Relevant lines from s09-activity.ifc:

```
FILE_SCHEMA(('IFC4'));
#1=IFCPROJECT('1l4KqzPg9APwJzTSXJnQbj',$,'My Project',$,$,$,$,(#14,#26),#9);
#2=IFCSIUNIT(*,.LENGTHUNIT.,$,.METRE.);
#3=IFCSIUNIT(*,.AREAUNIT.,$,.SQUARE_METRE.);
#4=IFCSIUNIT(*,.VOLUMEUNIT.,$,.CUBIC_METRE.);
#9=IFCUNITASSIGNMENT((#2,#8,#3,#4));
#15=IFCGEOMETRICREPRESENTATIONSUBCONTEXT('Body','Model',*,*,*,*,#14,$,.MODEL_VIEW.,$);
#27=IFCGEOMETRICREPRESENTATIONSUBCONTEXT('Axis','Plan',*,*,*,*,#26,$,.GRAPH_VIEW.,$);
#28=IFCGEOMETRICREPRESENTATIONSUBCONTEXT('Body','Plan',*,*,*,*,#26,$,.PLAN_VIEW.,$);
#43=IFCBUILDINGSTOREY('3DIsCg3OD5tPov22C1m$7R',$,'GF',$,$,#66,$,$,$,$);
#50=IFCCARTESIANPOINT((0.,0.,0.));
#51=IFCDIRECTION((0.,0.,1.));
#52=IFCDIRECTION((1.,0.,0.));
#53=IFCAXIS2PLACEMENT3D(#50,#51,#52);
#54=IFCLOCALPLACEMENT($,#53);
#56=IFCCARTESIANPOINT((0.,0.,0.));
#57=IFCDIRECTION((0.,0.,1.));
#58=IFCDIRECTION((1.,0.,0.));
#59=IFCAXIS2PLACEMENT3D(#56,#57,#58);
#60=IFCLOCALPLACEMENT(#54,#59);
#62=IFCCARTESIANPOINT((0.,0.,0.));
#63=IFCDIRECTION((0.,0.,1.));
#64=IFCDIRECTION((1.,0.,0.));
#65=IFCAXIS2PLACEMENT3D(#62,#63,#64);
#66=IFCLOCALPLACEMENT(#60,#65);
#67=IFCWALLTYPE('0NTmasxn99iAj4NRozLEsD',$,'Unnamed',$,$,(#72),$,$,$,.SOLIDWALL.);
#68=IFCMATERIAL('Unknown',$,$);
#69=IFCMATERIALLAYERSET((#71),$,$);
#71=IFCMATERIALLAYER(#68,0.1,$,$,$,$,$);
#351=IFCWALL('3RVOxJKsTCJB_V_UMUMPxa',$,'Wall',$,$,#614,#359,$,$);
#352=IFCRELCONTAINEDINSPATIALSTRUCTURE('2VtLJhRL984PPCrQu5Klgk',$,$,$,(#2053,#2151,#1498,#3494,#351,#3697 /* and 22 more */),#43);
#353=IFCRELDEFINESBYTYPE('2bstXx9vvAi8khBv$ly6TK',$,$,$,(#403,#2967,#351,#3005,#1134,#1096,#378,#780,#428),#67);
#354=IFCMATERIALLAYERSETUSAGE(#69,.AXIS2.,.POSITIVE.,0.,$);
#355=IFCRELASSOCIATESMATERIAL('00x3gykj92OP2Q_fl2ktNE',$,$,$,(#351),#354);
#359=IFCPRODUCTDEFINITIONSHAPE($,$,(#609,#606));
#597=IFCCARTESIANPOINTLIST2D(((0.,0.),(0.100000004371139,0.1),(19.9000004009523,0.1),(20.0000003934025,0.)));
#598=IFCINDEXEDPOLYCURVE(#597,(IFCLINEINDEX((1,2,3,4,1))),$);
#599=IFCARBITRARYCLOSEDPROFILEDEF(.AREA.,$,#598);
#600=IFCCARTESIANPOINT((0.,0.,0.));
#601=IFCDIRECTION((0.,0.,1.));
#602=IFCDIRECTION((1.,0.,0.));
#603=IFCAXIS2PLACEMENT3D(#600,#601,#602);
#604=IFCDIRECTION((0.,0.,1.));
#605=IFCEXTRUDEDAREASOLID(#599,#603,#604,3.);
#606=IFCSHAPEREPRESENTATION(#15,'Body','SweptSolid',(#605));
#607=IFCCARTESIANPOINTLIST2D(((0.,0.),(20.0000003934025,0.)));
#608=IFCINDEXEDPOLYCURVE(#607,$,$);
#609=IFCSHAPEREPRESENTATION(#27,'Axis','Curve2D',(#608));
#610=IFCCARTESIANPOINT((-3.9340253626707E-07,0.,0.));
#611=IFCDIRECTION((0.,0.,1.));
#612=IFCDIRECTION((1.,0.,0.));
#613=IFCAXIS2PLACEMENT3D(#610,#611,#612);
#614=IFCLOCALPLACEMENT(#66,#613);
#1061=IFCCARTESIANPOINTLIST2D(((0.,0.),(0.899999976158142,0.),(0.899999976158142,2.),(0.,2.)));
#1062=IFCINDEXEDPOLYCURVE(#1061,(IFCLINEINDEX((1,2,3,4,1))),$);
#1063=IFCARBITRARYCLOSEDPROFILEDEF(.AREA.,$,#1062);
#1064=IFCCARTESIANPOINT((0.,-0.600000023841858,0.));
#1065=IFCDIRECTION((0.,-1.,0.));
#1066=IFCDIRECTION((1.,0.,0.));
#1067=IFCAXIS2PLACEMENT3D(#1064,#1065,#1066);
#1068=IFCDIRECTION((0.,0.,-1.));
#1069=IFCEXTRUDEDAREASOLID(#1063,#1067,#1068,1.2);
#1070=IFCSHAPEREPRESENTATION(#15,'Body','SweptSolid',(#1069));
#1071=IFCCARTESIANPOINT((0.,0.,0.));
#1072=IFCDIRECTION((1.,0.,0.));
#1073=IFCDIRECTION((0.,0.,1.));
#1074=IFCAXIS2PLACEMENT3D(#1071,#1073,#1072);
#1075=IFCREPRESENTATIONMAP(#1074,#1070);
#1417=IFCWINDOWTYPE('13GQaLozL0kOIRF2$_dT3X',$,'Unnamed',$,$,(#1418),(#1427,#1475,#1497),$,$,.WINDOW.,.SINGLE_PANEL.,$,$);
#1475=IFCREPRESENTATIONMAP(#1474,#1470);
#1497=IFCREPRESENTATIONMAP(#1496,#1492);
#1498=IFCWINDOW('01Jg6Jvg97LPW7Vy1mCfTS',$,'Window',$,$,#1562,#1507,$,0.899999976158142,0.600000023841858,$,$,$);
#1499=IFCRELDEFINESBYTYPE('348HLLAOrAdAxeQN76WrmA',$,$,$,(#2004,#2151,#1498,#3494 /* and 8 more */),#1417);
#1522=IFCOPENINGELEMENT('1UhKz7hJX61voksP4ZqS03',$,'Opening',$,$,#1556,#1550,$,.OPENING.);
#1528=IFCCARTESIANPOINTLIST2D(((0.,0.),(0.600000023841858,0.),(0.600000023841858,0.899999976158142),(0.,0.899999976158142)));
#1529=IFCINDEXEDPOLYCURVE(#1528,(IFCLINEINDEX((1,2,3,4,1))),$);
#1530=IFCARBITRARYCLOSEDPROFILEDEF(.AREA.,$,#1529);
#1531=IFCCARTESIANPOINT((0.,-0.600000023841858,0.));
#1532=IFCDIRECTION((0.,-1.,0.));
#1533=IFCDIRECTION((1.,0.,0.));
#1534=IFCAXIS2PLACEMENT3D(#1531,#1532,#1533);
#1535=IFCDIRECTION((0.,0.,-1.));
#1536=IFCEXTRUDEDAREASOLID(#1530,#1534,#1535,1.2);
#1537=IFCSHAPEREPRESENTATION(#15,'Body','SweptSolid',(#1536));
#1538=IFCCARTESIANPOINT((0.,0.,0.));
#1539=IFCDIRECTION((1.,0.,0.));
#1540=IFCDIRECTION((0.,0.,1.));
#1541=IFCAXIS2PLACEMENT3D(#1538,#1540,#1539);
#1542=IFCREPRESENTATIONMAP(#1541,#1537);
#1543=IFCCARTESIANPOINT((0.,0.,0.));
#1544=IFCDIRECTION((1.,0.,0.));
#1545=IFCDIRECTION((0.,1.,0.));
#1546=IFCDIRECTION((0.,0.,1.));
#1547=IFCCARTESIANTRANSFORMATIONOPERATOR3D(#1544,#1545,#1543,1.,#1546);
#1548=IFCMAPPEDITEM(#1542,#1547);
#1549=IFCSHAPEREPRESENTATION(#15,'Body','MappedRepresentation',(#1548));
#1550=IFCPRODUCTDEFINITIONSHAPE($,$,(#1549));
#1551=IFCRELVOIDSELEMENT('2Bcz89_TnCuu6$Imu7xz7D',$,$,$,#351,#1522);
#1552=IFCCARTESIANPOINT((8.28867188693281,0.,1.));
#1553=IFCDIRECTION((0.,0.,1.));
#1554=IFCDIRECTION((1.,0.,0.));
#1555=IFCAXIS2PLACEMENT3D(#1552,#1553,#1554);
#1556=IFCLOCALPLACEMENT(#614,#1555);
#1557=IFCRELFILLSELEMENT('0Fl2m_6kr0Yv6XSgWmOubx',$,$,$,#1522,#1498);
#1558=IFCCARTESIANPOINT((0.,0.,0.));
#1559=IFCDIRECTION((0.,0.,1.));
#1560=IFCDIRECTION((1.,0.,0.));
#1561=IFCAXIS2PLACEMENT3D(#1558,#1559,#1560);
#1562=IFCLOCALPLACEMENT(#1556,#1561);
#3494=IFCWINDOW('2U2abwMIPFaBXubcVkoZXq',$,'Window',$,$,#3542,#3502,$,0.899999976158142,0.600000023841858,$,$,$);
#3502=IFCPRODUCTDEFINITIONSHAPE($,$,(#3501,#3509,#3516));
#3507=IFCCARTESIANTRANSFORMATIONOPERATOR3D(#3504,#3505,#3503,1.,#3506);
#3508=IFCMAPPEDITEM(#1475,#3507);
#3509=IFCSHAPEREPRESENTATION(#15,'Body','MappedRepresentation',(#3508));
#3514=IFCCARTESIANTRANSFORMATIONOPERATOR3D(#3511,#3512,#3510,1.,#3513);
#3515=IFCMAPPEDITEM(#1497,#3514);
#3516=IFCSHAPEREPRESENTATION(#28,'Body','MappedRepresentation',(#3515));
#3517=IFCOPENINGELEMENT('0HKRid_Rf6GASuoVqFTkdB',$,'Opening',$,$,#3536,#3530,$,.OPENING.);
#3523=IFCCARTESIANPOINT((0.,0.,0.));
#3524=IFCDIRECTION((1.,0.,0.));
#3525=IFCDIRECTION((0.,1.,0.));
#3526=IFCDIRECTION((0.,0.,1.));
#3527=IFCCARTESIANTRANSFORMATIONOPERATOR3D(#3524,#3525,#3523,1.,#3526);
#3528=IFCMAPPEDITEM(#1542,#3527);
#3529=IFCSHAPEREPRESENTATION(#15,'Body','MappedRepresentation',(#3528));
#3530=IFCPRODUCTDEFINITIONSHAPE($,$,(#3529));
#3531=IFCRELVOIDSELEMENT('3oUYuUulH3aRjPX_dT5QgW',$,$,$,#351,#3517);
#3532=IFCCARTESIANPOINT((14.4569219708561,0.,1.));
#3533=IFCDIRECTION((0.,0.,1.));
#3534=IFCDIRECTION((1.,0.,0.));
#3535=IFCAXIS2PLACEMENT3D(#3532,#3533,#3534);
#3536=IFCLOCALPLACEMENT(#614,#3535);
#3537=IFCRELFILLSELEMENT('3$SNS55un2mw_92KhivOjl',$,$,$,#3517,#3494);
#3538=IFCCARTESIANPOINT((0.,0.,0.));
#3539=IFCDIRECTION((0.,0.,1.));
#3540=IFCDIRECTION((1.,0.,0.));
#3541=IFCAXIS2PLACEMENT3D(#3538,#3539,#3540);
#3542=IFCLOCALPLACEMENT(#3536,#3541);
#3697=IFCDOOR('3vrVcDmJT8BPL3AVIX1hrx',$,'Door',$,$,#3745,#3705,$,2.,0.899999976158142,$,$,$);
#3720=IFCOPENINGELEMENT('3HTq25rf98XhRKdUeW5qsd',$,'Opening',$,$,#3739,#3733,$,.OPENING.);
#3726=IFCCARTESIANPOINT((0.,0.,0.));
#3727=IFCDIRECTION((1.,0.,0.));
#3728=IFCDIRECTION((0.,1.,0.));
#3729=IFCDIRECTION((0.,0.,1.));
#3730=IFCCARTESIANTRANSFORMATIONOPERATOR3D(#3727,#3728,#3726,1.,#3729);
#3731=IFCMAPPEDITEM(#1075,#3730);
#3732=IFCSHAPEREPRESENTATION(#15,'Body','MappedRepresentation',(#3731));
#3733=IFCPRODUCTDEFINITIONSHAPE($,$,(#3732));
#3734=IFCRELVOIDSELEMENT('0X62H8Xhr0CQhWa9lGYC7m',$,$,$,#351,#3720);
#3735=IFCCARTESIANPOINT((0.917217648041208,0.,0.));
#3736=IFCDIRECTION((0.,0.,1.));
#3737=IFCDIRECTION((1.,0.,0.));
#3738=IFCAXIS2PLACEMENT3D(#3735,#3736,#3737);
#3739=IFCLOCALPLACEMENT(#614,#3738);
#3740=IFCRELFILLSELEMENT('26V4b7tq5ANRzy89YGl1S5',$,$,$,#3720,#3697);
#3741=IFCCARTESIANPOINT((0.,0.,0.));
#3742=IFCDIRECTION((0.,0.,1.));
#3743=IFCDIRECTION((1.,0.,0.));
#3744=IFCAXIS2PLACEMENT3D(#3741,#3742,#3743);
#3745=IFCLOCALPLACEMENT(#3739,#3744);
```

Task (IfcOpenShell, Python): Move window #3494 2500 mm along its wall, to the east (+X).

```python
import ifcopenshell
import ifcopenshell.api.geometry
import ifcopenshell.util.placement
import ifcopenshell.util.unit

model = ifcopenshell.open("s09-activity.ifc")
unit_scale = ifcopenshell.util.unit.calculate_unit_scale(model)

window = model.by_guid("2U2abwMIPFaBXubcVkoZXq")
opening = window.FillsVoids[0].RelatingOpeningElement
wall = opening.VoidsElements[0].RelatingBuildingElement

wall_matrix = ifcopenshell.util.placement.get_local_placement(wall.ObjectPlacement)
shift = wall_matrix[:3, 0] * 2.5 / unit_scale
before = ifcopenshell.util.placement.get_local_placement(window.ObjectPlacement)[:3, 3].copy()

# The window is placed relative to its opening, so it follows when the opening moves.
matrix = ifcopenshell.util.placement.get_local_placement(opening.ObjectPlacement)
matrix[:3, 3] += shift
ifcopenshell.api.geometry.edit_object_placement(
    model, product=opening, matrix=matrix, is_si=False, should_transform_children=True
)

after = ifcopenshell.util.placement.get_local_placement(window.ObjectPlacement)[:3, 3]
print("window moved by", (after - before).round(3) + 0.0)

model.write("s09-activity_v2.ifc")
```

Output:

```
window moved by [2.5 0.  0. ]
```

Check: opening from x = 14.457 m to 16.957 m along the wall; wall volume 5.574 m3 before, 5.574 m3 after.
